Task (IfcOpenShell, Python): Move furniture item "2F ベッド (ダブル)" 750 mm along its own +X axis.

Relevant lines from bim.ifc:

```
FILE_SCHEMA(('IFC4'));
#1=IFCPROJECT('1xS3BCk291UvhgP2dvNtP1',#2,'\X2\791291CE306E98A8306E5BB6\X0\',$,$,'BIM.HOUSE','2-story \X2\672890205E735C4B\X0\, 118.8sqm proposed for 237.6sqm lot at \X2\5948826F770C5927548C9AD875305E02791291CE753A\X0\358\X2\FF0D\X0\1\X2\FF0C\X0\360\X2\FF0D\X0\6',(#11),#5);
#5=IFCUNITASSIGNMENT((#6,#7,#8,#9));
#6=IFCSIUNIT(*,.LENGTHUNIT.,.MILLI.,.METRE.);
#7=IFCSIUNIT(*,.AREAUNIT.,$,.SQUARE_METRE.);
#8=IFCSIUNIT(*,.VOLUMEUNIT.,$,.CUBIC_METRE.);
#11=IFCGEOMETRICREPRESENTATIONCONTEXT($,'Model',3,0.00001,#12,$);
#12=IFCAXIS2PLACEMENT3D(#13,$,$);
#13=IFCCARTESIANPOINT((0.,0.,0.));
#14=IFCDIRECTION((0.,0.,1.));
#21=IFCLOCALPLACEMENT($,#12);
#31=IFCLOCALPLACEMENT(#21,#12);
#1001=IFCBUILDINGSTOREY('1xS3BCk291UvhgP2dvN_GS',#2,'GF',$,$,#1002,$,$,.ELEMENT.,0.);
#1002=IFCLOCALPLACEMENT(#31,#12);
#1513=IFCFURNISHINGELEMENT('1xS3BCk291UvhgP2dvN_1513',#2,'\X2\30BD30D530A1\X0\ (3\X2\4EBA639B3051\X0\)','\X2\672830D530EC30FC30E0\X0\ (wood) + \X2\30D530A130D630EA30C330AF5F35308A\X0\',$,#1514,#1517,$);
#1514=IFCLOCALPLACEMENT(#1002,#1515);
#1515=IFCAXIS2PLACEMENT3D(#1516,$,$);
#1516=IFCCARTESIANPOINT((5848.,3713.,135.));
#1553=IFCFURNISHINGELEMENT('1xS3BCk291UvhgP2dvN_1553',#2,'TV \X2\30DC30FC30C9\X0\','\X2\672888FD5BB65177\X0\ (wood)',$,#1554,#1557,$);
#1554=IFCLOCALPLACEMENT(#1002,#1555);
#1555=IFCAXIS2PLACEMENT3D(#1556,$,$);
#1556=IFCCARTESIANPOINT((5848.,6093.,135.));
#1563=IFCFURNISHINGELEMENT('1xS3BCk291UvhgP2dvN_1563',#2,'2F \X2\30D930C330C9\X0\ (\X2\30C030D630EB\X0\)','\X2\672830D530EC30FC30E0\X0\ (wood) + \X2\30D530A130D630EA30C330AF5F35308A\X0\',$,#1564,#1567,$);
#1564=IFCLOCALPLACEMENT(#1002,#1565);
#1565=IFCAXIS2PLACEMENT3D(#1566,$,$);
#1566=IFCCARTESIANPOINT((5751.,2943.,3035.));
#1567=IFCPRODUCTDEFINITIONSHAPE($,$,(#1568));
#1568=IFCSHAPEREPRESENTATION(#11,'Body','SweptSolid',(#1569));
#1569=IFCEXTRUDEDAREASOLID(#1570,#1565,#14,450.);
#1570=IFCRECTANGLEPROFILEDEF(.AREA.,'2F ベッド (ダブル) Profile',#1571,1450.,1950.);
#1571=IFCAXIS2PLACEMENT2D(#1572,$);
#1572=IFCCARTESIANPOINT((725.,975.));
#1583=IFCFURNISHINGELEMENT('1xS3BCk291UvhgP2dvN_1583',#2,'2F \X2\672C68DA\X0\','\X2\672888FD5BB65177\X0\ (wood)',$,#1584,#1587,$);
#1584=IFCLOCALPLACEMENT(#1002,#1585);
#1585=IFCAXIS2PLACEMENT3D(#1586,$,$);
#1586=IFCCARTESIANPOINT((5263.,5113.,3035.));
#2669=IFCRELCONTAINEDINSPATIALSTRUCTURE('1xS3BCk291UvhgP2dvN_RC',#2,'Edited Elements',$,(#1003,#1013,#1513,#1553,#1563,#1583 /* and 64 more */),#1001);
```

```python
import ifcopenshell
import ifcopenshell.api.geometry
import ifcopenshell.util.placement
import ifcopenshell.util.unit

model = ifcopenshell.open("bim.ifc")
unit_scale = ifcopenshell.util.unit.calculate_unit_scale(model)

item = model.by_id(1563)
matrix = ifcopenshell.util.placement.get_local_placement(item.ObjectPlacement)
matrix[:3, 3] += matrix[:3, 0] * 0.75 / unit_scale
ifcopenshell.api.geometry.edit_object_placement(model, product=item, matrix=matrix, is_si=False)

print(ifcopenshell.util.placement.get_local_placement(item.ObjectPlacement).round(3) + 0.0)

model.write("bim_v2.ifc")
```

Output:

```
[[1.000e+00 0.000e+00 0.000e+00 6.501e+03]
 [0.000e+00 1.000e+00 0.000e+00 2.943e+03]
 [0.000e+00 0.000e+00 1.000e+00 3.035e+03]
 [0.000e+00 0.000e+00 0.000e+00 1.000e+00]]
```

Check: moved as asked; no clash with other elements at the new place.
